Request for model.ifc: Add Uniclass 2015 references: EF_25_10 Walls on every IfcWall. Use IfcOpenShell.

First a look at what the model holds.

```python
import ifcopenshell

model = ifcopenshell.open("model.ifc")
print(model.schema)
print("classifications:", [c.Name for c in model.by_type("IfcClassification")])
for ifc_class in ("IfcDoor", "IfcRoof", "IfcStair", "IfcWall", "IfcWindow"):
    print(ifc_class, len(model.by_type(ifc_class)))
```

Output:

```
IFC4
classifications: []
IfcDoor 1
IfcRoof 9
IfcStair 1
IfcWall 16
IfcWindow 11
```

```python
import ifcopenshell
import ifcopenshell.api.classification

model = ifcopenshell.open("model.ifc")

system = ifcopenshell.api.classification.add_classification(model, classification="Uniclass 2015")

codes = {
    "IfcWall": ("EF_25_10", "Walls"),
}
for ifc_class, (code, name) in codes.items():
    products = model.by_type(ifc_class)
    ifcopenshell.api.classification.add_reference(
        model, products=products, classification=system, identification=code, name=name
    )
    print(code, len(products))

model.write("model_v2.ifc")
```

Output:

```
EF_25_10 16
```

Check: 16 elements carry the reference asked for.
